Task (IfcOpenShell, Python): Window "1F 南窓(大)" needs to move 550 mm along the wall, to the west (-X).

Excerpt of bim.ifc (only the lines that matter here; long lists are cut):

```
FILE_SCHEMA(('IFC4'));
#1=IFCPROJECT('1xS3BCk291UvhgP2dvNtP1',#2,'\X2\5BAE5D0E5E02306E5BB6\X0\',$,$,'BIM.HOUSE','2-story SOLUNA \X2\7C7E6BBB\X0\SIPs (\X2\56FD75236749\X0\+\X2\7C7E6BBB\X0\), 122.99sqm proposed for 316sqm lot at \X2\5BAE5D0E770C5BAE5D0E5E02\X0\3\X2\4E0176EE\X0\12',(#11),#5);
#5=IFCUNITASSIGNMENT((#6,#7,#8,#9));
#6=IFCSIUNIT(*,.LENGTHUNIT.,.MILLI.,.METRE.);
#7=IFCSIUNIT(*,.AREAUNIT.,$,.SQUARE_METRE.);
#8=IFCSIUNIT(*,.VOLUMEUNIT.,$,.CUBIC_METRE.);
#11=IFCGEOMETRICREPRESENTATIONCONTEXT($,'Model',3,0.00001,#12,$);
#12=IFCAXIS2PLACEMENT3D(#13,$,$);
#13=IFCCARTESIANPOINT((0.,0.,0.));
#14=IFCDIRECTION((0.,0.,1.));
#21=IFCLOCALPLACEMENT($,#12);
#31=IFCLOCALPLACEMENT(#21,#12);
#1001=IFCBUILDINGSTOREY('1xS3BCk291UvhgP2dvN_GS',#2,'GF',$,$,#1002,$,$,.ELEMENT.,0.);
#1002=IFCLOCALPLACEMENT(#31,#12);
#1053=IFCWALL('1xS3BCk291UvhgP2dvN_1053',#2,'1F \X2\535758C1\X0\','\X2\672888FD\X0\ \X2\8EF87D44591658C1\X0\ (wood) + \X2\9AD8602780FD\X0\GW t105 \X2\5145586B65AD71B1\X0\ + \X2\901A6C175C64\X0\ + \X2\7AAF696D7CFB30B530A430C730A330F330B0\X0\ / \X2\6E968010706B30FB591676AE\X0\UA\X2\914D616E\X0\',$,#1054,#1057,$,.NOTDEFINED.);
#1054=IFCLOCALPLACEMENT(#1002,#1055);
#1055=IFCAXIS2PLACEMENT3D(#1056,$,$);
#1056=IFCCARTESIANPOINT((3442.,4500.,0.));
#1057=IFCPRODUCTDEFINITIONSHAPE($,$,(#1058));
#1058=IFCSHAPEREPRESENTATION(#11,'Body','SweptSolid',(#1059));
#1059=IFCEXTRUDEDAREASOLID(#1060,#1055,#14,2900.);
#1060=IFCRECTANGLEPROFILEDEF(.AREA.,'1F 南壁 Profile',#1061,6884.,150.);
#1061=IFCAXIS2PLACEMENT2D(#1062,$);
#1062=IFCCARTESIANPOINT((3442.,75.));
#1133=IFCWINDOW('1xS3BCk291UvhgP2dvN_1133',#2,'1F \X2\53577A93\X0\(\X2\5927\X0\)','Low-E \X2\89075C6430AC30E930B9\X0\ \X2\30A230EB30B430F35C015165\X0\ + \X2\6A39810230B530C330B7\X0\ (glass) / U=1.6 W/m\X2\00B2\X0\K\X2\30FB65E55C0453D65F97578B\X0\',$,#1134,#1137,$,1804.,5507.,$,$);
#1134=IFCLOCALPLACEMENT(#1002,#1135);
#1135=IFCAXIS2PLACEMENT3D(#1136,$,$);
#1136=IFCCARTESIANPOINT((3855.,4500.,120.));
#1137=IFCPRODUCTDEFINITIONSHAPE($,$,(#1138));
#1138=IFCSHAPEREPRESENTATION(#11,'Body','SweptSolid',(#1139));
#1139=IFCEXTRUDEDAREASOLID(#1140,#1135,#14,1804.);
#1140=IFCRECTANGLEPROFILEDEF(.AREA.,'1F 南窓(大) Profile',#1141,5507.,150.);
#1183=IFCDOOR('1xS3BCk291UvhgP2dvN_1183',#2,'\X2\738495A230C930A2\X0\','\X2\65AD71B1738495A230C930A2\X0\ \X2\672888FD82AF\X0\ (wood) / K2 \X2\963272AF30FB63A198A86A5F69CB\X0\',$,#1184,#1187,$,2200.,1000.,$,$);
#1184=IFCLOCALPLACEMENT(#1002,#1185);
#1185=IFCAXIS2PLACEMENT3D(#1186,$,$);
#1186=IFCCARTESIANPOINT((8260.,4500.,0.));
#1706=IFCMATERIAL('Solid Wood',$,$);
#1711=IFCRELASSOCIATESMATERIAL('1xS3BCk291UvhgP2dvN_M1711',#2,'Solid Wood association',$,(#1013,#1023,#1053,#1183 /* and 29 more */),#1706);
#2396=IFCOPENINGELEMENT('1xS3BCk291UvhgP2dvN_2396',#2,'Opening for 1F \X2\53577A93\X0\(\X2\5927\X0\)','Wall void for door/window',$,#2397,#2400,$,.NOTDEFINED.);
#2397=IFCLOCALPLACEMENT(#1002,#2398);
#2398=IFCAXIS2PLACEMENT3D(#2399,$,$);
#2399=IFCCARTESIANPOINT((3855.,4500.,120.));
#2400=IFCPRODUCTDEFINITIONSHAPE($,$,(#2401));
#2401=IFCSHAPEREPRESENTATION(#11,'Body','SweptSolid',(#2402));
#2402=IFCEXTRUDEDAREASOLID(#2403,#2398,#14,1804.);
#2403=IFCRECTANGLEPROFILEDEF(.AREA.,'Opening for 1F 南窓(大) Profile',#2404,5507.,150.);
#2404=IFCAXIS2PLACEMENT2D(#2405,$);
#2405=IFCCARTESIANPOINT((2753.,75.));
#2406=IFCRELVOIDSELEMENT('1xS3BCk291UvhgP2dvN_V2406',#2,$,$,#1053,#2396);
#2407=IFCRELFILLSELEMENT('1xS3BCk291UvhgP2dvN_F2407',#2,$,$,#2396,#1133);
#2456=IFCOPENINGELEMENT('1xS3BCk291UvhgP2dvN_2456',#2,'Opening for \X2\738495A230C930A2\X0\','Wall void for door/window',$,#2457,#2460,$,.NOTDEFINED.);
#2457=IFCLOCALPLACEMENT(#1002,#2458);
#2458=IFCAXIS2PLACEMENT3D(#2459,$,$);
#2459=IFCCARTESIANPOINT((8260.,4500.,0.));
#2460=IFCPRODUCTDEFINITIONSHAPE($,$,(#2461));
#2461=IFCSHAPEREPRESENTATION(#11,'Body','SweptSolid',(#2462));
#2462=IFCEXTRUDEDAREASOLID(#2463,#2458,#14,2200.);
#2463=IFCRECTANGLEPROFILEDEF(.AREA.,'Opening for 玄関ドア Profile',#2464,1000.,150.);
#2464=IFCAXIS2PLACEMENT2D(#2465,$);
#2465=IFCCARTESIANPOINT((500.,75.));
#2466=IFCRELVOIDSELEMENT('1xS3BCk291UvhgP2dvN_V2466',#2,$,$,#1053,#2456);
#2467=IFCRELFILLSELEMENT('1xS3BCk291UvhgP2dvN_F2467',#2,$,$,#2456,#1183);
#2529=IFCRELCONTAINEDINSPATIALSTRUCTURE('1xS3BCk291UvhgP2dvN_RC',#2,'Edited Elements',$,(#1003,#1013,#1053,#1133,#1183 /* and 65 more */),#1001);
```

```python
import ifcopenshell
import ifcopenshell.api.geometry
import ifcopenshell.util.placement
import ifcopenshell.util.unit

model = ifcopenshell.open("bim.ifc")
unit_scale = ifcopenshell.util.unit.calculate_unit_scale(model)

window = model.by_guid("1xS3BCk291UvhgP2dvN_1133")
opening = window.FillsVoids[0].RelatingOpeningElement
wall = opening.VoidsElements[0].RelatingBuildingElement

wall_matrix = ifcopenshell.util.placement.get_local_placement(wall.ObjectPlacement)
shift = wall_matrix[:3, 0] * -0.55 / unit_scale
before = ifcopenshell.util.placement.get_local_placement(window.ObjectPlacement)[:3, 3].copy()

# The window is not placed relative to its opening, so move both.
for product in (opening, window):
    matrix = ifcopenshell.util.placement.get_local_placement(product.ObjectPlacement)
    matrix[:3, 3] += shift
    ifcopenshell.api.geometry.edit_object_placement(model, product=product, matrix=matrix, is_si=False)

after = ifcopenshell.util.placement.get_local_placement(window.ObjectPlacement)[:3, 3]
print("window moved by", (after - before).round(3) + 0.0)

model.write("bim_edited.ifc")
```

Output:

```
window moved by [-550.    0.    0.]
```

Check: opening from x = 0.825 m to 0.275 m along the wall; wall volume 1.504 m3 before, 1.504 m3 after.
